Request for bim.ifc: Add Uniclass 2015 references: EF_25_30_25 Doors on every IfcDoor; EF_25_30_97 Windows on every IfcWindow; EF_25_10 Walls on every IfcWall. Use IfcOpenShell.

First a look at what the model holds.

```python
import ifcopenshell

model = ifcopenshell.open("bim.ifc")
print(model.schema)
print("classifications:", [c.Name for c in model.by_type("IfcClassification")])
for ifc_class in ("IfcDoor", "IfcRoof", "IfcStair", "IfcWall", "IfcWindow"):
    print(ifc_class, len(model.by_type(ifc_class)))
```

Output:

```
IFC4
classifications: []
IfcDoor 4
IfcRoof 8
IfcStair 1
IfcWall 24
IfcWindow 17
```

```python
import ifcopenshell
import ifcopenshell.api.classification

model = ifcopenshell.open("bim.ifc")

system = ifcopenshell.api.classification.add_classification(model, classification="Uniclass 2015")

codes = {
    "IfcDoor": ("EF_25_30_25", "Doors"),
    "IfcWindow": ("EF_25_30_97", "Windows"),
    "IfcWall": ("EF_25_10", "Walls"),
}
for ifc_class, (code, name) in codes.items():
    products = model.by_type(ifc_class)
    ifcopenshell.api.classification.add_reference(
        model, products=products, classification=system, identification=code, name=name
    )
    print(code, len(products))

model.write("bim_v2.ifc")
```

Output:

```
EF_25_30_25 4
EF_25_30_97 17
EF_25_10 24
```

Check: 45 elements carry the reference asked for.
